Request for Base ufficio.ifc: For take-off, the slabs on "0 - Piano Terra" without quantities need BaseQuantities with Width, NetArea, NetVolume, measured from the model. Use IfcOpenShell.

First a look at what the model holds.

```python
import ifcopenshell
import ifcopenshell.util.element
import ifcopenshell.util.unit

model = ifcopenshell.open("Base ufficio.ifc")
print(model.schema)
for unit_type in ("LENGTHUNIT", "AREAUNIT", "VOLUMEUNIT"):
    print(unit_type, ifcopenshell.util.unit.calculate_unit_scale(model, unit_type))
storey = next(s for s in model.by_type("IfcBuildingStorey") if s.Name == "0 - Piano Terra")
slabs = [e for e in ifcopenshell.util.element.get_decomposition(storey) if e.is_a("IfcSlab")]
for e in sorted(slabs, key=lambda e: e.id()):
    print(e.id(), e.is_a(), e.Name, list(ifcopenshell.util.element.get_psets(e, qtos_only=True)), sep=" | ")
```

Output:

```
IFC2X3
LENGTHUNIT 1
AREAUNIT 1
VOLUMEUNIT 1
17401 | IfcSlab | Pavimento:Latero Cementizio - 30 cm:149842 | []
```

```python
import ifcopenshell
import ifcopenshell.api.pset
import ifcopenshell.geom
import ifcopenshell.util.element
import ifcopenshell.util.shape
import ifcopenshell.util.unit

model = ifcopenshell.open("Base ufficio.ifc")
unit_scale = ifcopenshell.util.unit.calculate_unit_scale(model)
area_scale = ifcopenshell.util.unit.calculate_unit_scale(model, "AREAUNIT")
volume_scale = ifcopenshell.util.unit.calculate_unit_scale(model, "VOLUMEUNIT")
settings = ifcopenshell.geom.settings()

storey = next(s for s in model.by_type("IfcBuildingStorey") if s.Name == "0 - Piano Terra")
slabs = [e for e in ifcopenshell.util.element.get_decomposition(storey) if e.is_a("IfcSlab")]

for e in sorted(slabs, key=lambda e: e.id()):
    if ifcopenshell.util.element.get_psets(e, qtos_only=True, should_inherit=False):
        continue
    # Geometry comes back in metres, in the element's own axes.
    shape = ifcopenshell.geom.create_shape(settings, e)
    values = {
        "Width": ifcopenshell.util.shape.get_z(shape.geometry) / unit_scale,
        "NetArea": ifcopenshell.util.shape.get_footprint_area(shape.geometry) / area_scale,
        "NetVolume": ifcopenshell.util.shape.get_volume(shape.geometry) / volume_scale,
    }
    qto = ifcopenshell.api.pset.add_qto(model, product=e, name="BaseQuantities")
    ifcopenshell.api.pset.edit_qto(model, qto=qto, properties=values)
    print(e.id(), {k: round(v, 3) for k, v in values.items()})

model.write("Base ufficio_edited.ifc")
```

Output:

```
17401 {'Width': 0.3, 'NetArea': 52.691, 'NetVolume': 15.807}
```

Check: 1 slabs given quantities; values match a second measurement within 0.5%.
